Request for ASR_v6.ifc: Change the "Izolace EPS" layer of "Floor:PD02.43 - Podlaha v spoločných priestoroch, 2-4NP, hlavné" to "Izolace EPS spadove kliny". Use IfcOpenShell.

First a look at what the model holds.

```python
import ifcopenshell
import ifcopenshell.util.element

model = ifcopenshell.open("ASR_v6.ifc")
print(model.schema)
for layer_set in model.by_type("IfcMaterialLayerSet"):
    if layer_set.LayerSetName == "Floor:PD02.43 - Podlaha v spoločných priestoroch, 2-4NP, hlavné":
        for layer in layer_set.MaterialLayers:
            print(layer.id(), layer.Material and layer.Material.Name, layer.LayerThickness, sep=" | ")
        print(len(ifcopenshell.util.element.get_elements_by_material(model, layer_set)), "elements and types use it")
print(sorted(m.Name for m in model.by_type("IfcMaterial") if m.Name)[:60])
```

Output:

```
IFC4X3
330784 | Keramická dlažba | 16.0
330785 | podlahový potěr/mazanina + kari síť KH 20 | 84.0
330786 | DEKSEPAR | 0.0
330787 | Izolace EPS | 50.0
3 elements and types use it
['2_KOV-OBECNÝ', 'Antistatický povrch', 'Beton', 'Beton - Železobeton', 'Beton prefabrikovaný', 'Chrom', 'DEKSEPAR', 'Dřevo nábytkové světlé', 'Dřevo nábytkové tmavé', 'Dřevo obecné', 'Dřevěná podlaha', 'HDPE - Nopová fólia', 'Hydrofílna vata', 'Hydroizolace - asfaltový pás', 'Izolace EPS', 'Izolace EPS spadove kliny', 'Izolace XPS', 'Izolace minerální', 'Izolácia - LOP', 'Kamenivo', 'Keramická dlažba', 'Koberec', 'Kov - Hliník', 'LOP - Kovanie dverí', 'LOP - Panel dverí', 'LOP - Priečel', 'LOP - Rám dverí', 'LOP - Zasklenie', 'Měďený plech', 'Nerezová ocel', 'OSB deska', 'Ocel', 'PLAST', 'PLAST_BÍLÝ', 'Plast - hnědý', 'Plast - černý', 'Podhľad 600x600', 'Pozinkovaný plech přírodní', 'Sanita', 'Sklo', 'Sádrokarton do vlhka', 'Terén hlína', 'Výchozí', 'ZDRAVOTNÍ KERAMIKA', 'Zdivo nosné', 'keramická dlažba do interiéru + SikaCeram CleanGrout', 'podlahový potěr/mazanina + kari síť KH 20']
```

```python
import ifcopenshell
import ifcopenshell.api.material

model = ifcopenshell.open("ASR_v6.ifc")

layer_set = next(s for s in model.by_type("IfcMaterialLayerSet") if s.LayerSetName == "Floor:PD02.43 - Podlaha v spoločných priestoroch, 2-4NP, hlavné")
layer = next(l for l in layer_set.MaterialLayers if l.Material and l.Material.Name == "Izolace EPS")
material = next(m for m in model.by_type("IfcMaterial") if m.Name == "Izolace EPS spadove kliny")

# Point this one layer at the other material; renaming the old one would change it everywhere.
ifcopenshell.api.material.edit_layer(model, layer=layer, attributes={"Name": material.Name}, material=material)

print([l.Material.Name if l.Material else None for l in layer_set.MaterialLayers])

model.write("ASR_v6_updated.ifc")
```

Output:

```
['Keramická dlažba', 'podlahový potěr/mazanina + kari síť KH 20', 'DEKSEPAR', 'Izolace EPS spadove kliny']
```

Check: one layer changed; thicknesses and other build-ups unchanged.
